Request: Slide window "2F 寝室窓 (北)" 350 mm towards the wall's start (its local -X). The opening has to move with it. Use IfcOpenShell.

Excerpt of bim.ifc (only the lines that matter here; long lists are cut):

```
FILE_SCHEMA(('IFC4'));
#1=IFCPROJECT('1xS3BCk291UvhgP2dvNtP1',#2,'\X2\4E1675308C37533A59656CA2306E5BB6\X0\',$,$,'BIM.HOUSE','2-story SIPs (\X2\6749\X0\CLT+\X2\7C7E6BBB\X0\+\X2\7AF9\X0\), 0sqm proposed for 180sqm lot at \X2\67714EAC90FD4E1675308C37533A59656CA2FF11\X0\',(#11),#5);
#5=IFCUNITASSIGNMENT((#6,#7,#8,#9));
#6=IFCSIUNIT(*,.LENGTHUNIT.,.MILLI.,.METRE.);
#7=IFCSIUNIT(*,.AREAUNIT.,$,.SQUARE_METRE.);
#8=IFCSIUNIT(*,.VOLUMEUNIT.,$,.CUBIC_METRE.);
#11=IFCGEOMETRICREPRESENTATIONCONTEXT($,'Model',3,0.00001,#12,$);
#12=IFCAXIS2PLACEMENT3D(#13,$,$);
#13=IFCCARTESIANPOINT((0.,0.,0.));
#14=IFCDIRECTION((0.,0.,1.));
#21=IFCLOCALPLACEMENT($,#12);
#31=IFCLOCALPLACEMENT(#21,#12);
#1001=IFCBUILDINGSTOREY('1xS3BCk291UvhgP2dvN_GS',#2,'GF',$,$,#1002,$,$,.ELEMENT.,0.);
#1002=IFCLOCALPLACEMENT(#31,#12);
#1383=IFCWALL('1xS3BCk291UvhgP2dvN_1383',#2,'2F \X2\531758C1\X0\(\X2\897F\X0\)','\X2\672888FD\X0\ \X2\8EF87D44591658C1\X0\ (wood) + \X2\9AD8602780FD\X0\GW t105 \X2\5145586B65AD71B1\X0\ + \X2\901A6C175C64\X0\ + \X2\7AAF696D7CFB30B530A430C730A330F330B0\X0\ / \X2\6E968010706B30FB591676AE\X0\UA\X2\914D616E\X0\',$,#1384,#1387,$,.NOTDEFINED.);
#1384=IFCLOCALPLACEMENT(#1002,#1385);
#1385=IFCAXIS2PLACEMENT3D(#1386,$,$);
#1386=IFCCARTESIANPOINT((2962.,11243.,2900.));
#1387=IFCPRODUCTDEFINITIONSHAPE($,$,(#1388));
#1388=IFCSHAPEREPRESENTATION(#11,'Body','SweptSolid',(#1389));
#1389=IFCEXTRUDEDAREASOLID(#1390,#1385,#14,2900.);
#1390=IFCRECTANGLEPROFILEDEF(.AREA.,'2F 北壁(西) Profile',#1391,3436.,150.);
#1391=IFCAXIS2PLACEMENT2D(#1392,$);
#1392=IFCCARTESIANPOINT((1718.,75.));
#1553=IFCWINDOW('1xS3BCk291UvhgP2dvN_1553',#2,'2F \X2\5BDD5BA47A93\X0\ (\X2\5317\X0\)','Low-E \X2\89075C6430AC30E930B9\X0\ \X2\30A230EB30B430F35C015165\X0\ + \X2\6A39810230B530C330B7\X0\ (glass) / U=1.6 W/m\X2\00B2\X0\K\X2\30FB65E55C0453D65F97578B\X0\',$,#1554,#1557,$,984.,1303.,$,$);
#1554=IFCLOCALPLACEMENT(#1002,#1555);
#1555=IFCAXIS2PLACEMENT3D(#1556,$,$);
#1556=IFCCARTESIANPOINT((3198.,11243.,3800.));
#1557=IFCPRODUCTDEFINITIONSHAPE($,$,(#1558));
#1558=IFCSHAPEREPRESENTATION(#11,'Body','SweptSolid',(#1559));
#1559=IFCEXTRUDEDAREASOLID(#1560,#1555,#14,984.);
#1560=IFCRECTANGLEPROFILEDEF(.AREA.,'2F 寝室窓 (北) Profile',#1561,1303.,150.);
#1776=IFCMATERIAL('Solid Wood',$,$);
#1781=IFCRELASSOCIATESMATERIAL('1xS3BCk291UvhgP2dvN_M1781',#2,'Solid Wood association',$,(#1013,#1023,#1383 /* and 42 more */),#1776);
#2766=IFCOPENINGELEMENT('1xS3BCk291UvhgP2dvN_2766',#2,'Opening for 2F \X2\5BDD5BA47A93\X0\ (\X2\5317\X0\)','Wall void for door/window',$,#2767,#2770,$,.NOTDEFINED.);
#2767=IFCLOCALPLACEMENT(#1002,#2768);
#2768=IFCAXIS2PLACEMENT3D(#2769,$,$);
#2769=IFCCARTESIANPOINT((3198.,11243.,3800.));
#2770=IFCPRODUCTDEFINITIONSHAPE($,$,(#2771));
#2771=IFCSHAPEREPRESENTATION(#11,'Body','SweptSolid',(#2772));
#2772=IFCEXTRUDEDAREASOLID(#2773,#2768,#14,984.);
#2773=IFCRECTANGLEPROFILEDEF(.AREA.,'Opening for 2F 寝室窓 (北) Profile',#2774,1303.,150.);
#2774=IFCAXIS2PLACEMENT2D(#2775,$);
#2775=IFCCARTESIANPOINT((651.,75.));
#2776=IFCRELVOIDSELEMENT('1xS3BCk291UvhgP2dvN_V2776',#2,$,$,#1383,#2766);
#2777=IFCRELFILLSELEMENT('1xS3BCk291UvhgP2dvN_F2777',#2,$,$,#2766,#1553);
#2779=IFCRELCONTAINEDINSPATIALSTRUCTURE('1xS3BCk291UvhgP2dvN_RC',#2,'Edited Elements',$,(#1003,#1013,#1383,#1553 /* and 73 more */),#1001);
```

```python
import ifcopenshell
import ifcopenshell.api.geometry
import ifcopenshell.util.placement
import ifcopenshell.util.unit

model = ifcopenshell.open("bim.ifc")
unit_scale = ifcopenshell.util.unit.calculate_unit_scale(model)

window = model.by_guid("1xS3BCk291UvhgP2dvN_1553")
opening = window.FillsVoids[0].RelatingOpeningElement
wall = opening.VoidsElements[0].RelatingBuildingElement

wall_matrix = ifcopenshell.util.placement.get_local_placement(wall.ObjectPlacement)
shift = wall_matrix[:3, 0] * -0.35 / unit_scale
before = ifcopenshell.util.placement.get_local_placement(window.ObjectPlacement)[:3, 3].copy()

# The window is not placed relative to its opening, so move both.
for product in (opening, window):
    matrix = ifcopenshell.util.placement.get_local_placement(product.ObjectPlacement)
    matrix[:3, 3] += shift
    ifcopenshell.api.geometry.edit_object_placement(model, product=product, matrix=matrix, is_si=False)

after = ifcopenshell.util.placement.get_local_placement(window.ObjectPlacement)[:3, 3]
print("window moved by", (after - before).round(3) + 0.0)

model.write("bim_rev.ifc")
```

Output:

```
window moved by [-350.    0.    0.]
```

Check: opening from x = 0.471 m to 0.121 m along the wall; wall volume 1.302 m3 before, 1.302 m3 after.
